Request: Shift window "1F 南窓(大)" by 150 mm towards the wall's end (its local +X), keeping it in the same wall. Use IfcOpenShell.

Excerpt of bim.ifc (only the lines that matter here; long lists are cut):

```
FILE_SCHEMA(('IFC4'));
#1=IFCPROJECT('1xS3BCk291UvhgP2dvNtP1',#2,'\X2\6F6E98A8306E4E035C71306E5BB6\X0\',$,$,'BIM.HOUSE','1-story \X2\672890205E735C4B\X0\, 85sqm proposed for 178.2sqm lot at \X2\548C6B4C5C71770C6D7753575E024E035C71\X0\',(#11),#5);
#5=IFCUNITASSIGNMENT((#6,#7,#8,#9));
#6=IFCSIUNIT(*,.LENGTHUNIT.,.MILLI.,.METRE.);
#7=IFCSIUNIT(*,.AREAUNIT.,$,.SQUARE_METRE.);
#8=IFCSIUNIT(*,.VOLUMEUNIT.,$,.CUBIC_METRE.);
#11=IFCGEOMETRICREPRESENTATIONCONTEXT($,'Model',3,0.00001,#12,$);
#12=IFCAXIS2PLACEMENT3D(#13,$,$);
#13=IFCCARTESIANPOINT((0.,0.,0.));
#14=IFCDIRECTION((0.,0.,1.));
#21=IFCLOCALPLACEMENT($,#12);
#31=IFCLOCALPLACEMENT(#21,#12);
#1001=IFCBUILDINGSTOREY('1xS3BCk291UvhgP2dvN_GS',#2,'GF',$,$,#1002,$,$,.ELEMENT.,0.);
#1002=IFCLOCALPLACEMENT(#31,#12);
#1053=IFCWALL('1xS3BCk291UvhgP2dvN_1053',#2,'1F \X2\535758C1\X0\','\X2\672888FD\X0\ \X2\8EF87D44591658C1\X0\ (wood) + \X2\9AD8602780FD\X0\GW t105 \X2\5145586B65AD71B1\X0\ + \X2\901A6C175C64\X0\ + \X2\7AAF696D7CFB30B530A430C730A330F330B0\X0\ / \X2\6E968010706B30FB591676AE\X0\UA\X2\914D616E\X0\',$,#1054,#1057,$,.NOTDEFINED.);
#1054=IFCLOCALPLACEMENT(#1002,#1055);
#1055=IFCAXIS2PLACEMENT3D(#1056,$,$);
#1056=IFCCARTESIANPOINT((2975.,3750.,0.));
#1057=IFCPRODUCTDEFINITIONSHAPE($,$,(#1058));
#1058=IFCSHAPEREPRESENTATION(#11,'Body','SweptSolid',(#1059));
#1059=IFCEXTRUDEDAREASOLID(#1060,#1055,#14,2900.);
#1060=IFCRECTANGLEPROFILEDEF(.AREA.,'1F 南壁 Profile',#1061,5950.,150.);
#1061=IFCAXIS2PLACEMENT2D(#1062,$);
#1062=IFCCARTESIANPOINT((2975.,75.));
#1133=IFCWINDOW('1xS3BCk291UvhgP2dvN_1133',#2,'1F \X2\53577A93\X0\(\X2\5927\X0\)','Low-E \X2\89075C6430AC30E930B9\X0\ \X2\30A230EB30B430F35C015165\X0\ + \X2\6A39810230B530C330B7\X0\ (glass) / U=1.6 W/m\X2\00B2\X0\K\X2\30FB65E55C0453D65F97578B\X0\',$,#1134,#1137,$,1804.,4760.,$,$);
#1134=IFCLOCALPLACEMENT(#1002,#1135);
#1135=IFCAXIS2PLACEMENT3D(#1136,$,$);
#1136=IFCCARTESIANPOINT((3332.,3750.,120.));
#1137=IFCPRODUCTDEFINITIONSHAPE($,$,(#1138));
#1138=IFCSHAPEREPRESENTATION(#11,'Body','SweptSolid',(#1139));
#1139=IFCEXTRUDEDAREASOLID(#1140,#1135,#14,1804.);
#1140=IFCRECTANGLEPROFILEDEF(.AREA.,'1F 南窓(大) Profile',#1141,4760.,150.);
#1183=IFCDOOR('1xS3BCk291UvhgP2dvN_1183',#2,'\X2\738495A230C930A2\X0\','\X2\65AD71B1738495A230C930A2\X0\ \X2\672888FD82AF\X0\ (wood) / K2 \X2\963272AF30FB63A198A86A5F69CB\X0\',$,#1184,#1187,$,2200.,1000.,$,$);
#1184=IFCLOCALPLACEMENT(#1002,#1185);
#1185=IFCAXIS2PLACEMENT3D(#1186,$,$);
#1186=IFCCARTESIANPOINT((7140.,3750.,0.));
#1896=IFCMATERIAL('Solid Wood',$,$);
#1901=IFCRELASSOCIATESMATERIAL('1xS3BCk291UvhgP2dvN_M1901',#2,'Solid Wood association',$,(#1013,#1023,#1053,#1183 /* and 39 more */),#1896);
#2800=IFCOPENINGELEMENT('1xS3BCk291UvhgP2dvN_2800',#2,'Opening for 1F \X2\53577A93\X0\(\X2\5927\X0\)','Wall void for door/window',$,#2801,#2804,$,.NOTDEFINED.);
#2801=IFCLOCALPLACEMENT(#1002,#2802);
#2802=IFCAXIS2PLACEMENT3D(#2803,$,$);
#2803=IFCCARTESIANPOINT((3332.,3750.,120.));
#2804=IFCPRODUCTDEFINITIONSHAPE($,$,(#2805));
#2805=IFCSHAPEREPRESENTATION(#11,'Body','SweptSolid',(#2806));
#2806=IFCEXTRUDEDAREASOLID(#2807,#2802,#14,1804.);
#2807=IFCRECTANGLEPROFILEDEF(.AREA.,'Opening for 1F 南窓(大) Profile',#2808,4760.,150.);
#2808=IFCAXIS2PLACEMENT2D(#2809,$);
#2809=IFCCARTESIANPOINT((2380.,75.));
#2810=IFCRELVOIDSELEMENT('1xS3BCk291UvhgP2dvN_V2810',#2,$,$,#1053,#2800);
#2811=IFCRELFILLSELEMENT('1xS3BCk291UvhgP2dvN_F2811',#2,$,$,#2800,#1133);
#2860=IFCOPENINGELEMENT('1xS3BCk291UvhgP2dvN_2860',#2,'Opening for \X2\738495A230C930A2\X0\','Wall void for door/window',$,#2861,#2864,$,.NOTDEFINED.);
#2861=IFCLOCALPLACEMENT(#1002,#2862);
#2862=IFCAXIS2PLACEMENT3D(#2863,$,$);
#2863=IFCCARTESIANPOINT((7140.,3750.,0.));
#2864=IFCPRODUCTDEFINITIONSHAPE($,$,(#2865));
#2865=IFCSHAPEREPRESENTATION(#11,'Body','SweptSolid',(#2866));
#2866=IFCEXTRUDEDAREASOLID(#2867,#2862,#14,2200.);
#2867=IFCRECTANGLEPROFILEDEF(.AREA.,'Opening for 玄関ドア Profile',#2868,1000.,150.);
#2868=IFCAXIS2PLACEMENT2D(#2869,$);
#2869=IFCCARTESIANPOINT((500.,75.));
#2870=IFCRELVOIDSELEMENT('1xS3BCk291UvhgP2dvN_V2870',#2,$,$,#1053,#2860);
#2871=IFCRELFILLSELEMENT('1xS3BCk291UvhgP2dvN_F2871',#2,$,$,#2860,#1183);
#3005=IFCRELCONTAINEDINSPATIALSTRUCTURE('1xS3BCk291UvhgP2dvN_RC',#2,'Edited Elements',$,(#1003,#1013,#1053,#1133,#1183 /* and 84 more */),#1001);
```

```python
import ifcopenshell
import ifcopenshell.api.geometry
import ifcopenshell.util.placement

model = ifcopenshell.open("bim.ifc")

window = model.by_guid("1xS3BCk291UvhgP2dvN_1133")
opening = window.FillsVoids[0].RelatingOpeningElement
wall = opening.VoidsElements[0].RelatingBuildingElement

wall_matrix = ifcopenshell.util.placement.get_local_placement(wall.ObjectPlacement)
shift = wall_matrix[:3, 0] * 150.0
before = ifcopenshell.util.placement.get_local_placement(window.ObjectPlacement)[:3, 3].copy()

# The window is not placed relative to its opening, so move both.
for product in (opening, window):
    matrix = ifcopenshell.util.placement.get_local_placement(product.ObjectPlacement)
    matrix[:3, 3] += shift
    ifcopenshell.api.geometry.edit_object_placement(model, product=product, matrix=matrix, is_si=False)

after = ifcopenshell.util.placement.get_local_placement(window.ObjectPlacement)[:3, 3]
print("window moved by", (after - before).round(3) + 0.0)

model.write("bim_v2.ifc")
```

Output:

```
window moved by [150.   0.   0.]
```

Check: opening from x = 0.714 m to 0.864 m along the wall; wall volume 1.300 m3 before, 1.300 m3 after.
